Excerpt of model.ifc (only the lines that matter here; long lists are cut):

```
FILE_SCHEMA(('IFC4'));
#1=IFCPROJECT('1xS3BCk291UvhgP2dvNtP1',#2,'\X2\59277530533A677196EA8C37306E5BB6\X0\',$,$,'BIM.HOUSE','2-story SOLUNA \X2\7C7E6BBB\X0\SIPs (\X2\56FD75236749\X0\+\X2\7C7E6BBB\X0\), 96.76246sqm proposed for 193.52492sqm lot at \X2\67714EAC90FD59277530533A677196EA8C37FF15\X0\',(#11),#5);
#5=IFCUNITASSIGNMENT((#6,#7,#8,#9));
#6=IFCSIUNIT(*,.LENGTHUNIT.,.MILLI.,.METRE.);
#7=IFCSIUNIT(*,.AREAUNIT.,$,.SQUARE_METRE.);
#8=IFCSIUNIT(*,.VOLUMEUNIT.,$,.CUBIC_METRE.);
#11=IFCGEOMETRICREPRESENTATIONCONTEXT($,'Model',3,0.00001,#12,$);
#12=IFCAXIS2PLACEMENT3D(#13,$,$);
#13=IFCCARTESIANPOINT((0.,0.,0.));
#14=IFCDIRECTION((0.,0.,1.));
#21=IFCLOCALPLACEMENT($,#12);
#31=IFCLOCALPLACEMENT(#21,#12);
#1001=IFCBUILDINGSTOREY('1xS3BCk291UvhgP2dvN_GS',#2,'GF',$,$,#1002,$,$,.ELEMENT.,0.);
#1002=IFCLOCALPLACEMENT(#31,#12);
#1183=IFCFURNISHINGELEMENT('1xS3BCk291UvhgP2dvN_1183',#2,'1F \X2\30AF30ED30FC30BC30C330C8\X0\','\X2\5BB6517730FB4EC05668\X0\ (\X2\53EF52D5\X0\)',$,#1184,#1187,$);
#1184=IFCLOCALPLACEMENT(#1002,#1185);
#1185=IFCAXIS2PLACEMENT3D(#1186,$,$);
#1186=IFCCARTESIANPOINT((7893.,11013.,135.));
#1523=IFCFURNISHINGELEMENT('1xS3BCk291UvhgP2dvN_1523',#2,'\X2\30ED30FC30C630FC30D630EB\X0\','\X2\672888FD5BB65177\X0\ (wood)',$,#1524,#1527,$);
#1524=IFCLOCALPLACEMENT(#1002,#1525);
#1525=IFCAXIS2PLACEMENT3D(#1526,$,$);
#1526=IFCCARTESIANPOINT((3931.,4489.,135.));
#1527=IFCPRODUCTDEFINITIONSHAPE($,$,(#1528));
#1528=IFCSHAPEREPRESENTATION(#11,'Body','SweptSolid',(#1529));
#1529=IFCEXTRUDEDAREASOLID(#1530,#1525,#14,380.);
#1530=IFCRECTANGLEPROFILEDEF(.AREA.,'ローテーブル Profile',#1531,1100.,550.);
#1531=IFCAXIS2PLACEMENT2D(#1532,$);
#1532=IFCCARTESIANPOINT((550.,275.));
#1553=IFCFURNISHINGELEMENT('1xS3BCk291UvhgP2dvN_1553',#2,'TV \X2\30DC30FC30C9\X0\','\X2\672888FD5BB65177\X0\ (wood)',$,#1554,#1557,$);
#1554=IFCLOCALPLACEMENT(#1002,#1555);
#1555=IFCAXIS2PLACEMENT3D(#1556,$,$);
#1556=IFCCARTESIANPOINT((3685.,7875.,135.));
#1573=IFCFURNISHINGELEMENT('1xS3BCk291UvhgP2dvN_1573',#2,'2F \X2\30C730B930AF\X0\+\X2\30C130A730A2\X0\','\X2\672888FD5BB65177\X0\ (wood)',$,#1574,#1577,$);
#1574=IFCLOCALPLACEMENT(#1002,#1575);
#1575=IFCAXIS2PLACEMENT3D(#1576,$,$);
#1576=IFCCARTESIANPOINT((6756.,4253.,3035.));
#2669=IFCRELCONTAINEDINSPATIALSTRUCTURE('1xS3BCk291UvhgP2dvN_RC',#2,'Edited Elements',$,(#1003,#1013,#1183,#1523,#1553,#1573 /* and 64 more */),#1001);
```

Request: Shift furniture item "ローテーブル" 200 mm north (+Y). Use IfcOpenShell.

```python
import ifcopenshell
import ifcopenshell.api.geometry
import ifcopenshell.util.placement
import ifcopenshell.util.unit

model = ifcopenshell.open("model.ifc")
unit_scale = ifcopenshell.util.unit.calculate_unit_scale(model)

item = model.by_id(1523)
matrix = ifcopenshell.util.placement.get_local_placement(item.ObjectPlacement)
matrix[1, 3] += 0.2 / unit_scale
ifcopenshell.api.geometry.edit_object_placement(model, product=item, matrix=matrix, is_si=False)

print(ifcopenshell.util.placement.get_local_placement(item.ObjectPlacement).round(3) + 0.0)

model.write("model_updated.ifc")
```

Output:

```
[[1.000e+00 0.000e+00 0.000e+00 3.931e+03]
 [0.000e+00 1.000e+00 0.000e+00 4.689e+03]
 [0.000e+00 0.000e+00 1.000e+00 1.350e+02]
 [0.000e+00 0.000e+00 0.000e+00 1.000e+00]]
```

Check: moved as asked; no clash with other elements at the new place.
